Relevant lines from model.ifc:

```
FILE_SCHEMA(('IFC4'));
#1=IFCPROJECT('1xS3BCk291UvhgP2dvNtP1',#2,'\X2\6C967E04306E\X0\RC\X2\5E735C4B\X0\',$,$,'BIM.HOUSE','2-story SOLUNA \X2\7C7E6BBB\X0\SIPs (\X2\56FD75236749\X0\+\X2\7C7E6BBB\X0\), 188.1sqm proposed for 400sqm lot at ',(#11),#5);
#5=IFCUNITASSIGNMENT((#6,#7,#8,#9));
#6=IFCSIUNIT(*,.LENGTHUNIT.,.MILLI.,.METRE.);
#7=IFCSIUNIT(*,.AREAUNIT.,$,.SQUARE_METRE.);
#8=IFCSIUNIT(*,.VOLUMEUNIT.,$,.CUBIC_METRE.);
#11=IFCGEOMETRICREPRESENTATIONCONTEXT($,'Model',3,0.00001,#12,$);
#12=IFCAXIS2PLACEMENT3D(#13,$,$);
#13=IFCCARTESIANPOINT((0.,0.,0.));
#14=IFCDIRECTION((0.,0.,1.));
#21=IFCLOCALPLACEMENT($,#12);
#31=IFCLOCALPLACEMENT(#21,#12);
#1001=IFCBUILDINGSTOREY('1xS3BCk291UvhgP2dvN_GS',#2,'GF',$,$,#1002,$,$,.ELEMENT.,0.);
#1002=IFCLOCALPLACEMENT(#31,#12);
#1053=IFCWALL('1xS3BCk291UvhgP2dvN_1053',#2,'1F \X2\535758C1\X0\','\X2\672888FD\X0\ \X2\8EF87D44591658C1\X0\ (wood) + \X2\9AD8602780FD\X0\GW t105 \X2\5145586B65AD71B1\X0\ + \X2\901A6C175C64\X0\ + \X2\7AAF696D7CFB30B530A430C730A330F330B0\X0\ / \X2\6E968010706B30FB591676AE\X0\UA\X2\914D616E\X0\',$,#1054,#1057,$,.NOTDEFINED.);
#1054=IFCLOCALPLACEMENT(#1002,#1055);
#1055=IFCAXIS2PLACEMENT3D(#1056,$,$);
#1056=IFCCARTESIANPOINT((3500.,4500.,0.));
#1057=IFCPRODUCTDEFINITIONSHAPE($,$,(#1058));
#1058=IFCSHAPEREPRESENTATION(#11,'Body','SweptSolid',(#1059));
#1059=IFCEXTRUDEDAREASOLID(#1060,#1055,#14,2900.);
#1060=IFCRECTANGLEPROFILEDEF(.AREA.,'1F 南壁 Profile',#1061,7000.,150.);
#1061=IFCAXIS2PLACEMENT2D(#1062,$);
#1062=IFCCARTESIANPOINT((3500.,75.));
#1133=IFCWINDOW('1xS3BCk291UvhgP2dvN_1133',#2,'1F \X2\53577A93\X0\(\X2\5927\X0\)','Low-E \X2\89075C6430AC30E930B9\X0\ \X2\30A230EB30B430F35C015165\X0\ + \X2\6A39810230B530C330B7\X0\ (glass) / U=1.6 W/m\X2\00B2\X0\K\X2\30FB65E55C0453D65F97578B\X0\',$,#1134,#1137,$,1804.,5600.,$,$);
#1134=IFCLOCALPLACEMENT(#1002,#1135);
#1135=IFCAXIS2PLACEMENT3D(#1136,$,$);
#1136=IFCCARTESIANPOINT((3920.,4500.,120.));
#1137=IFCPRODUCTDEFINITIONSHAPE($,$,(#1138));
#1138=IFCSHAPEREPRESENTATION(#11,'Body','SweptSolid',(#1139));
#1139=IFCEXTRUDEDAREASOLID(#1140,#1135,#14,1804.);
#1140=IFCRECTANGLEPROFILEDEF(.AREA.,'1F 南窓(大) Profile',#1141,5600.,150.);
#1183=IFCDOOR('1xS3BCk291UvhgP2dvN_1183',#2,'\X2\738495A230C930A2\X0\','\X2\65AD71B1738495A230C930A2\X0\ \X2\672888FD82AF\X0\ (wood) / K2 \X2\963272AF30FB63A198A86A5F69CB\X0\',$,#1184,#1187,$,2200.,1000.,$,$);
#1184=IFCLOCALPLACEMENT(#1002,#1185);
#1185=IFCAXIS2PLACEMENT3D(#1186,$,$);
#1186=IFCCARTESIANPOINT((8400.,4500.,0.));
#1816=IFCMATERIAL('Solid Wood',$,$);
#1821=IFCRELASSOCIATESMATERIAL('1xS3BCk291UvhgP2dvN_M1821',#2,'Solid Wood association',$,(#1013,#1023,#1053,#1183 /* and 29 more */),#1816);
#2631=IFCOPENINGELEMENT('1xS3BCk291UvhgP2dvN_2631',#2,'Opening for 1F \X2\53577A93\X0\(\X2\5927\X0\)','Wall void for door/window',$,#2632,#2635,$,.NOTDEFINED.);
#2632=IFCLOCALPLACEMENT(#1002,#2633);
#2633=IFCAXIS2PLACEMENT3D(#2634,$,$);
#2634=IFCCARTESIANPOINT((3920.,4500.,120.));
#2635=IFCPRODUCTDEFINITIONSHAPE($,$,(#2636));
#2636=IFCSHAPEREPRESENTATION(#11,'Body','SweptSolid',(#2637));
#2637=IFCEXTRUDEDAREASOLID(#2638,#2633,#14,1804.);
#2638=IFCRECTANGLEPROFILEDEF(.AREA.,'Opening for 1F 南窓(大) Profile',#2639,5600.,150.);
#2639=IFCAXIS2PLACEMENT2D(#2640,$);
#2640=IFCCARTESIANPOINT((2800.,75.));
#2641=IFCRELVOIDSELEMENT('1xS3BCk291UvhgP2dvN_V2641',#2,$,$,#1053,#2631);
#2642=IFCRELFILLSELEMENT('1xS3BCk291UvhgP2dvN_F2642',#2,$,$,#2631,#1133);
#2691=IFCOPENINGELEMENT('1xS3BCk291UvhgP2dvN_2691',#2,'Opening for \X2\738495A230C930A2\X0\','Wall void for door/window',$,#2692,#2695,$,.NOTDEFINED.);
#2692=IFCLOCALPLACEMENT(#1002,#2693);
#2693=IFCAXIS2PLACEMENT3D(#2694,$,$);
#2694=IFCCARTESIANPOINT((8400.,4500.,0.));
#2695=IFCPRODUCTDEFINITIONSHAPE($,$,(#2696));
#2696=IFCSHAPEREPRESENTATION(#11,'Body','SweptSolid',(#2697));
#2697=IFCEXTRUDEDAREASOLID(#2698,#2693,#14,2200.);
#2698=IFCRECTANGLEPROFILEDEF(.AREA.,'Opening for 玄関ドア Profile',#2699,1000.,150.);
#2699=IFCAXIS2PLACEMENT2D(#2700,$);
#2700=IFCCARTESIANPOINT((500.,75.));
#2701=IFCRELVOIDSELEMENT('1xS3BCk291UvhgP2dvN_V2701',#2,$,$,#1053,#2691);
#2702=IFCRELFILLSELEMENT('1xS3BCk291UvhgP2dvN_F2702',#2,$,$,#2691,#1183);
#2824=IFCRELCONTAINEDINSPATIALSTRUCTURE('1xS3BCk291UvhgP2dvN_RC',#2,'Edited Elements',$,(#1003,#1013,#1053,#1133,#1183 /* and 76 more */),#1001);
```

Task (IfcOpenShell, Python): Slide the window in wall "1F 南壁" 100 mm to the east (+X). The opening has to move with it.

```python
import ifcopenshell
import ifcopenshell.api.geometry
import ifcopenshell.util.placement

model = ifcopenshell.open("model.ifc")

window = model.by_id(1133)
opening = window.FillsVoids[0].RelatingOpeningElement
wall = opening.VoidsElements[0].RelatingBuildingElement

wall_matrix = ifcopenshell.util.placement.get_local_placement(wall.ObjectPlacement)
shift = wall_matrix[:3, 0] * 100.0
before = ifcopenshell.util.placement.get_local_placement(window.ObjectPlacement)[:3, 3].copy()

# The window is not placed relative to its opening, so move both.
for product in (opening, window):
    matrix = ifcopenshell.util.placement.get_local_placement(product.ObjectPlacement)
    matrix[:3, 3] += shift
    ifcopenshell.api.geometry.edit_object_placement(model, product=product, matrix=matrix, is_si=False)

after = ifcopenshell.util.placement.get_local_placement(window.ObjectPlacement)[:3, 3]
print("window moved by", (after - before).round(3) + 0.0)

model.write("model_v2.ifc")
```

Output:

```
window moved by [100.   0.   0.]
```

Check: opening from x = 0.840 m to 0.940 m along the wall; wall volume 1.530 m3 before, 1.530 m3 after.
